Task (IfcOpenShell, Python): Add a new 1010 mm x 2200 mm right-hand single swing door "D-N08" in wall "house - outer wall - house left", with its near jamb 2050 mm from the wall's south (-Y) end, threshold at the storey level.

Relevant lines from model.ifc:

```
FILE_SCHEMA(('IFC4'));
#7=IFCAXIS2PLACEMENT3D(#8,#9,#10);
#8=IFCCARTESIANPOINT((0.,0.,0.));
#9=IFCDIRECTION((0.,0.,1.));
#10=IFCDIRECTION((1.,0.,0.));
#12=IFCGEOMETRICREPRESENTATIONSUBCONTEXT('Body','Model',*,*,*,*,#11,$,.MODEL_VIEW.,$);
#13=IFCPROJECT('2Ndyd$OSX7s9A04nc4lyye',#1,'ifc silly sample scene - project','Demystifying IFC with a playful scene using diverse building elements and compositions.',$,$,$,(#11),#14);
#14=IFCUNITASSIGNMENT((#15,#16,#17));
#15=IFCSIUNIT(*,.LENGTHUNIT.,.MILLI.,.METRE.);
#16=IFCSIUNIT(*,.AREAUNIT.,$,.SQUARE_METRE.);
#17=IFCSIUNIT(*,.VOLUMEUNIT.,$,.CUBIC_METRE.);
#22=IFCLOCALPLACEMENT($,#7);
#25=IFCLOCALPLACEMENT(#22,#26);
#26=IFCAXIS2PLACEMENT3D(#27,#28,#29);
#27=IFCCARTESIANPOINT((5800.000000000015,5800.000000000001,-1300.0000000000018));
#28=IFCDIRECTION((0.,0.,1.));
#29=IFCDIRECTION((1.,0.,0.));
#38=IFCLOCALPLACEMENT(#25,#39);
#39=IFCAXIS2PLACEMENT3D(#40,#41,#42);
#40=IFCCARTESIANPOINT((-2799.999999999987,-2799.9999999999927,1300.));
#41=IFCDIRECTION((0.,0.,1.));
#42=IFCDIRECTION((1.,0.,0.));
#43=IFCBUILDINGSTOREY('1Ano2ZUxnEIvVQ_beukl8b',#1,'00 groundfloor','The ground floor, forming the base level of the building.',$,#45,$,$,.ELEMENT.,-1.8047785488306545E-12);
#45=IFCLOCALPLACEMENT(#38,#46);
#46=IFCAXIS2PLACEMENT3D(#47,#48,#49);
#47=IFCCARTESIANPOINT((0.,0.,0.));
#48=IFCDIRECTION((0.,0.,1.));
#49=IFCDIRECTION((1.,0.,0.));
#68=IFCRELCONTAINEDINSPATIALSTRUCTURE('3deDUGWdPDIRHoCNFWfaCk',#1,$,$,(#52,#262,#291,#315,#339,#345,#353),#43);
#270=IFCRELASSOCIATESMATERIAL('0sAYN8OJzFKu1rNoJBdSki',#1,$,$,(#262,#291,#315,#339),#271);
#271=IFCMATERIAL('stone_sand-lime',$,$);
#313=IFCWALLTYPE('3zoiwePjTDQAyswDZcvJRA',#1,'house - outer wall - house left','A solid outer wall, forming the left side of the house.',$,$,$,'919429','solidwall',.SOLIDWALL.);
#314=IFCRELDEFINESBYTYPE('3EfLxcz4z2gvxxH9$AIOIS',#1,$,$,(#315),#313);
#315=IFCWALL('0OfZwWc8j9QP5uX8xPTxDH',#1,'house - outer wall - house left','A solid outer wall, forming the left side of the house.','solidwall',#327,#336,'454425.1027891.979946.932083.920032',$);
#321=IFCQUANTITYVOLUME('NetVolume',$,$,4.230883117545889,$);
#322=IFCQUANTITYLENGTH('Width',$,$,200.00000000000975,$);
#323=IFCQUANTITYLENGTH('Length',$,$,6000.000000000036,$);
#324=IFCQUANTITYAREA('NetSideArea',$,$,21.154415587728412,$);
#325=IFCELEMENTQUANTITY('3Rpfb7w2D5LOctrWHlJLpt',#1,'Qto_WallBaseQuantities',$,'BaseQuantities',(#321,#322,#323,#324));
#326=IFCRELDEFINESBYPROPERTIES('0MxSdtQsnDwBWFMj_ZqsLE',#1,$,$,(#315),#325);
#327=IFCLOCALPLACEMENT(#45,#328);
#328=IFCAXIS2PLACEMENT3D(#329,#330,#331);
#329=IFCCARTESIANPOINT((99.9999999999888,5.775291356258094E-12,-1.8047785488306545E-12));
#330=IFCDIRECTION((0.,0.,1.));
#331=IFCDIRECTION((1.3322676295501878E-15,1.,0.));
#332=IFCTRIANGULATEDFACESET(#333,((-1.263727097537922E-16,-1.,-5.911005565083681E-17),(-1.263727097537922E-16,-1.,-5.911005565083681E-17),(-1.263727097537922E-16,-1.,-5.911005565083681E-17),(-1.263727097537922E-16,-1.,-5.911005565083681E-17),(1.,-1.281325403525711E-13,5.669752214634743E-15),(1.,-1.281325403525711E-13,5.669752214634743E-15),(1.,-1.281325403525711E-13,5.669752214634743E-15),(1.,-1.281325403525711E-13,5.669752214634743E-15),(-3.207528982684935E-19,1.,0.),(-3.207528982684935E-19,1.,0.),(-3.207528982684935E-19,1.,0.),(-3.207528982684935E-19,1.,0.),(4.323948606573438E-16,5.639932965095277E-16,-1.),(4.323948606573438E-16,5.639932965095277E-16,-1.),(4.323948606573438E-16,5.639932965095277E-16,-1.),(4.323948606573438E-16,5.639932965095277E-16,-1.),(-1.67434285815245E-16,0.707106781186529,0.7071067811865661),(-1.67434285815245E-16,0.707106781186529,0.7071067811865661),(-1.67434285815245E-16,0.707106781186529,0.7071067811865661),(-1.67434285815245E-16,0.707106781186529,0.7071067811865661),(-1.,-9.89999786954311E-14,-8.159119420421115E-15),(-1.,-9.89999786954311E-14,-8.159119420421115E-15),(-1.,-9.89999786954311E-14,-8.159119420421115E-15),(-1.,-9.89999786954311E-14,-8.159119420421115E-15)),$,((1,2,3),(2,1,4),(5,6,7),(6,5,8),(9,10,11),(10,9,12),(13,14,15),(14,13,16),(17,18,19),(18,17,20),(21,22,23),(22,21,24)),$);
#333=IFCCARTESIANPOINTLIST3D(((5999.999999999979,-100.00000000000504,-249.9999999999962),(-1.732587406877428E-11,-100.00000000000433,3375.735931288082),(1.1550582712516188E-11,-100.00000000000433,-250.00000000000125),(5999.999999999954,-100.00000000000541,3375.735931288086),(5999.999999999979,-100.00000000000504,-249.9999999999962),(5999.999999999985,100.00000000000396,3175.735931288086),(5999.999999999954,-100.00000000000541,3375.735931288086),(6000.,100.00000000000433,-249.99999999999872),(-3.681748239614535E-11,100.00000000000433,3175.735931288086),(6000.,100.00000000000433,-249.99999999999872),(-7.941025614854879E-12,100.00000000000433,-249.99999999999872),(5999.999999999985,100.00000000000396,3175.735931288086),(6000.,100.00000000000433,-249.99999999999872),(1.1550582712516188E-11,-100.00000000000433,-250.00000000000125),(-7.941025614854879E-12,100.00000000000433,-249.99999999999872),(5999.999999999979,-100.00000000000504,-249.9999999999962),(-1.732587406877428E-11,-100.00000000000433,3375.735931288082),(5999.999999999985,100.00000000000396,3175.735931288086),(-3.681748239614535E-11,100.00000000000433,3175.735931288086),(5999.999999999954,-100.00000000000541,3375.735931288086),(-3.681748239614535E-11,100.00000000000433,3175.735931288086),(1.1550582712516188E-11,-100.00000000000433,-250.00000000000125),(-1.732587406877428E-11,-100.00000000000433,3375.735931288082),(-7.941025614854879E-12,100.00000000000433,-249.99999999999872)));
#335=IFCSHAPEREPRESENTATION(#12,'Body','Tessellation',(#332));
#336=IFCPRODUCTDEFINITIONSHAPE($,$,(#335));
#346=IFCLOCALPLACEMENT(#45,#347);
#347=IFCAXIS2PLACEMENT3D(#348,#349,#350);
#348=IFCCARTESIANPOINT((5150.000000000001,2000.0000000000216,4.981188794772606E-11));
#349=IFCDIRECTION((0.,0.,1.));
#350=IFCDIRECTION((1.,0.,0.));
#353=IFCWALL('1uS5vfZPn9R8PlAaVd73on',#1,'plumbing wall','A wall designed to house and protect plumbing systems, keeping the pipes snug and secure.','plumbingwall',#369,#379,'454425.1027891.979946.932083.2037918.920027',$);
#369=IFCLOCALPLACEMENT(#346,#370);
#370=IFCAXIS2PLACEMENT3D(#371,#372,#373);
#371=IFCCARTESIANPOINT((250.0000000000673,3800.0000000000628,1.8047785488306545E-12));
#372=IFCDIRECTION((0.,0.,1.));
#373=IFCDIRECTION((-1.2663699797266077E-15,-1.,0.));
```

```python
import numpy as np
import ifcopenshell
import ifcopenshell.api.feature
import ifcopenshell.api.geometry
import ifcopenshell.api.pset
import ifcopenshell.api.root
import ifcopenshell.api.spatial
import ifcopenshell.geom
import ifcopenshell.util.element
import ifcopenshell.util.placement
import ifcopenshell.util.representation
import ifcopenshell.util.shape
import ifcopenshell.util.unit

model = ifcopenshell.open("model.ifc")
unit_scale = ifcopenshell.util.unit.calculate_unit_scale(model)
area_scale = ifcopenshell.util.unit.calculate_unit_scale(model, "AREAUNIT")
volume_scale = ifcopenshell.util.unit.calculate_unit_scale(model, "VOLUMEUNIT")
settings = ifcopenshell.geom.settings()


def volume(element):
    """Net volume in cubic metres, openings subtracted."""
    shape = ifcopenshell.geom.create_shape(settings, element)
    return ifcopenshell.util.shape.get_volume(shape.geometry)


wall = model.by_id(315)
storey = ifcopenshell.util.element.get_container(wall, ifc_class="IfcBuildingStorey")
context = ifcopenshell.util.representation.get_context(model, "Model", "Body", "MODEL_VIEW")
before = volume(wall)

width, height, from_end, sill = 1.01, 2.2, 2.05, 0.0  # metres

# The wall runs along its own X axis, and the end named is its -X end.
wall_shape = ifcopenshell.geom.create_shape(settings, wall)
x, y, z = ifcopenshell.util.shape.get_vertices(wall_shape.geometry).T
start = x.min() + from_end
face, thickness = float(y.min()), float(y.max() - y.min())
wall_matrix = ifcopenshell.util.placement.get_local_placement(wall.ObjectPlacement)
level = ifcopenshell.util.placement.get_local_placement(storey.ObjectPlacement)[2, 3]


def in_wall(x, y):
    """Placement at x, y metres in the wall's axes, at sill height."""
    matrix = wall_matrix.copy()
    matrix[:, 3] = wall_matrix @ np.array([x / unit_scale, y / unit_scale, 0.0, 1.0])
    matrix[2, 3] = level + sill / unit_scale
    return matrix


# Opening: a box that overshoots both wall faces by 50 mm.
opening = ifcopenshell.api.root.create_entity(model, ifc_class="IfcOpeningElement", predefined_type="OPENING")
box = ifcopenshell.api.geometry.add_wall_representation(
    model, context=context, length=width, height=height, thickness=thickness + 0.1
)
ifcopenshell.api.geometry.assign_representation(model, product=opening, representation=box)
ifcopenshell.api.geometry.edit_object_placement(model, product=opening, matrix=in_wall(start, face - 0.05), is_si=False)
ifcopenshell.api.feature.add_feature(model, feature=opening, element=wall)

door = ifcopenshell.api.root.create_entity(model, ifc_class="IfcDoor", name="D-N08", predefined_type="DOOR")
door.OverallWidth, door.OverallHeight = width / unit_scale, height / unit_scale
door.OperationType = "SINGLE_SWING_RIGHT"
body = ifcopenshell.api.geometry.add_door_representation(
    model,
    context=context,
    overall_width=door.OverallWidth,
    overall_height=door.OverallHeight,
    operation_type="SINGLE_SWING_RIGHT",
    lining_properties={"LiningDepth": thickness / unit_scale, "ThresholdDepth": thickness / unit_scale},
)
ifcopenshell.api.geometry.assign_representation(model, product=door, representation=body)
ifcopenshell.api.spatial.assign_container(model, products=[door], relating_structure=storey)
ifcopenshell.api.feature.add_filling(model, opening=opening, element=door)

# The lining spans the wall, so the door starts at the wall face.
ifcopenshell.api.geometry.edit_object_placement(model, product=door, matrix=in_wall(start, face), is_si=False)

after = volume(wall)

# Update the wall's stored quantities.
qto = model.by_id(ifcopenshell.util.element.get_pset(wall, "Qto_WallBaseQuantities", should_inherit=False)["id"])
ifcopenshell.api.pset.edit_qto(model, qto=qto, properties={
    "NetVolume": after / volume_scale,
    "NetSideArea": after / thickness / area_scale,
})

print(f"wall volume {before:.3f} -> {after:.3f} m3")

model.write("model_v2.ifc")
```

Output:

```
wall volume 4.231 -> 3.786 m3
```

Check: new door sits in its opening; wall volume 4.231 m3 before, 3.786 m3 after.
